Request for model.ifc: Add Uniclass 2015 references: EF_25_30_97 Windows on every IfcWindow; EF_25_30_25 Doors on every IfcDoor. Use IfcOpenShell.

First a look at what the model holds.

```python
import ifcopenshell

model = ifcopenshell.open("model.ifc")
print(model.schema)
print("classifications:", [c.Name for c in model.by_type("IfcClassification")])
for ifc_class in ("IfcDoor", "IfcRoof", "IfcStair", "IfcWall", "IfcWindow"):
    print(ifc_class, len(model.by_type(ifc_class)))
```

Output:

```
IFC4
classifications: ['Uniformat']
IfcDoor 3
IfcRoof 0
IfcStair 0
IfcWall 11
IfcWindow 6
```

```python
import ifcopenshell
import ifcopenshell.api.classification

model = ifcopenshell.open("model.ifc")

system = ifcopenshell.api.classification.add_classification(model, classification="Uniclass 2015")

codes = {
    "IfcWindow": ("EF_25_30_97", "Windows"),
    "IfcDoor": ("EF_25_30_25", "Doors"),
}
for ifc_class, (code, name) in codes.items():
    products = model.by_type(ifc_class)
    ifcopenshell.api.classification.add_reference(
        model, products=products, classification=system, identification=code, name=name
    )
    print(code, len(products))

model.write("model_edited.ifc")
```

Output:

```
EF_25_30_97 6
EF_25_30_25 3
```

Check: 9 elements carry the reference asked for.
